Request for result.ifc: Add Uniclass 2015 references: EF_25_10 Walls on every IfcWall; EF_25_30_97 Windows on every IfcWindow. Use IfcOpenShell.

First a look at what the model holds.

```python
import ifcopenshell

model = ifcopenshell.open("result.ifc")
print(model.schema)
print("classifications:", [c.Name for c in model.by_type("IfcClassification")])
for ifc_class in ("IfcDoor", "IfcRoof", "IfcStair", "IfcWall", "IfcWindow"):
    print(ifc_class, len(model.by_type(ifc_class)))
```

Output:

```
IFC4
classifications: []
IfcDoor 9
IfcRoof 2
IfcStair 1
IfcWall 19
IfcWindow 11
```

```python
import ifcopenshell
import ifcopenshell.api.classification

model = ifcopenshell.open("result.ifc")

system = ifcopenshell.api.classification.add_classification(model, classification="Uniclass 2015")

codes = {
    "IfcWall": ("EF_25_10", "Walls"),
    "IfcWindow": ("EF_25_30_97", "Windows"),
}
for ifc_class, (code, name) in codes.items():
    products = model.by_type(ifc_class)
    ifcopenshell.api.classification.add_reference(
        model, products=products, classification=system, identification=code, name=name
    )
    print(code, len(products))

model.write("result_edited.ifc")
```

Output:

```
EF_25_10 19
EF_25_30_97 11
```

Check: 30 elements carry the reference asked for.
